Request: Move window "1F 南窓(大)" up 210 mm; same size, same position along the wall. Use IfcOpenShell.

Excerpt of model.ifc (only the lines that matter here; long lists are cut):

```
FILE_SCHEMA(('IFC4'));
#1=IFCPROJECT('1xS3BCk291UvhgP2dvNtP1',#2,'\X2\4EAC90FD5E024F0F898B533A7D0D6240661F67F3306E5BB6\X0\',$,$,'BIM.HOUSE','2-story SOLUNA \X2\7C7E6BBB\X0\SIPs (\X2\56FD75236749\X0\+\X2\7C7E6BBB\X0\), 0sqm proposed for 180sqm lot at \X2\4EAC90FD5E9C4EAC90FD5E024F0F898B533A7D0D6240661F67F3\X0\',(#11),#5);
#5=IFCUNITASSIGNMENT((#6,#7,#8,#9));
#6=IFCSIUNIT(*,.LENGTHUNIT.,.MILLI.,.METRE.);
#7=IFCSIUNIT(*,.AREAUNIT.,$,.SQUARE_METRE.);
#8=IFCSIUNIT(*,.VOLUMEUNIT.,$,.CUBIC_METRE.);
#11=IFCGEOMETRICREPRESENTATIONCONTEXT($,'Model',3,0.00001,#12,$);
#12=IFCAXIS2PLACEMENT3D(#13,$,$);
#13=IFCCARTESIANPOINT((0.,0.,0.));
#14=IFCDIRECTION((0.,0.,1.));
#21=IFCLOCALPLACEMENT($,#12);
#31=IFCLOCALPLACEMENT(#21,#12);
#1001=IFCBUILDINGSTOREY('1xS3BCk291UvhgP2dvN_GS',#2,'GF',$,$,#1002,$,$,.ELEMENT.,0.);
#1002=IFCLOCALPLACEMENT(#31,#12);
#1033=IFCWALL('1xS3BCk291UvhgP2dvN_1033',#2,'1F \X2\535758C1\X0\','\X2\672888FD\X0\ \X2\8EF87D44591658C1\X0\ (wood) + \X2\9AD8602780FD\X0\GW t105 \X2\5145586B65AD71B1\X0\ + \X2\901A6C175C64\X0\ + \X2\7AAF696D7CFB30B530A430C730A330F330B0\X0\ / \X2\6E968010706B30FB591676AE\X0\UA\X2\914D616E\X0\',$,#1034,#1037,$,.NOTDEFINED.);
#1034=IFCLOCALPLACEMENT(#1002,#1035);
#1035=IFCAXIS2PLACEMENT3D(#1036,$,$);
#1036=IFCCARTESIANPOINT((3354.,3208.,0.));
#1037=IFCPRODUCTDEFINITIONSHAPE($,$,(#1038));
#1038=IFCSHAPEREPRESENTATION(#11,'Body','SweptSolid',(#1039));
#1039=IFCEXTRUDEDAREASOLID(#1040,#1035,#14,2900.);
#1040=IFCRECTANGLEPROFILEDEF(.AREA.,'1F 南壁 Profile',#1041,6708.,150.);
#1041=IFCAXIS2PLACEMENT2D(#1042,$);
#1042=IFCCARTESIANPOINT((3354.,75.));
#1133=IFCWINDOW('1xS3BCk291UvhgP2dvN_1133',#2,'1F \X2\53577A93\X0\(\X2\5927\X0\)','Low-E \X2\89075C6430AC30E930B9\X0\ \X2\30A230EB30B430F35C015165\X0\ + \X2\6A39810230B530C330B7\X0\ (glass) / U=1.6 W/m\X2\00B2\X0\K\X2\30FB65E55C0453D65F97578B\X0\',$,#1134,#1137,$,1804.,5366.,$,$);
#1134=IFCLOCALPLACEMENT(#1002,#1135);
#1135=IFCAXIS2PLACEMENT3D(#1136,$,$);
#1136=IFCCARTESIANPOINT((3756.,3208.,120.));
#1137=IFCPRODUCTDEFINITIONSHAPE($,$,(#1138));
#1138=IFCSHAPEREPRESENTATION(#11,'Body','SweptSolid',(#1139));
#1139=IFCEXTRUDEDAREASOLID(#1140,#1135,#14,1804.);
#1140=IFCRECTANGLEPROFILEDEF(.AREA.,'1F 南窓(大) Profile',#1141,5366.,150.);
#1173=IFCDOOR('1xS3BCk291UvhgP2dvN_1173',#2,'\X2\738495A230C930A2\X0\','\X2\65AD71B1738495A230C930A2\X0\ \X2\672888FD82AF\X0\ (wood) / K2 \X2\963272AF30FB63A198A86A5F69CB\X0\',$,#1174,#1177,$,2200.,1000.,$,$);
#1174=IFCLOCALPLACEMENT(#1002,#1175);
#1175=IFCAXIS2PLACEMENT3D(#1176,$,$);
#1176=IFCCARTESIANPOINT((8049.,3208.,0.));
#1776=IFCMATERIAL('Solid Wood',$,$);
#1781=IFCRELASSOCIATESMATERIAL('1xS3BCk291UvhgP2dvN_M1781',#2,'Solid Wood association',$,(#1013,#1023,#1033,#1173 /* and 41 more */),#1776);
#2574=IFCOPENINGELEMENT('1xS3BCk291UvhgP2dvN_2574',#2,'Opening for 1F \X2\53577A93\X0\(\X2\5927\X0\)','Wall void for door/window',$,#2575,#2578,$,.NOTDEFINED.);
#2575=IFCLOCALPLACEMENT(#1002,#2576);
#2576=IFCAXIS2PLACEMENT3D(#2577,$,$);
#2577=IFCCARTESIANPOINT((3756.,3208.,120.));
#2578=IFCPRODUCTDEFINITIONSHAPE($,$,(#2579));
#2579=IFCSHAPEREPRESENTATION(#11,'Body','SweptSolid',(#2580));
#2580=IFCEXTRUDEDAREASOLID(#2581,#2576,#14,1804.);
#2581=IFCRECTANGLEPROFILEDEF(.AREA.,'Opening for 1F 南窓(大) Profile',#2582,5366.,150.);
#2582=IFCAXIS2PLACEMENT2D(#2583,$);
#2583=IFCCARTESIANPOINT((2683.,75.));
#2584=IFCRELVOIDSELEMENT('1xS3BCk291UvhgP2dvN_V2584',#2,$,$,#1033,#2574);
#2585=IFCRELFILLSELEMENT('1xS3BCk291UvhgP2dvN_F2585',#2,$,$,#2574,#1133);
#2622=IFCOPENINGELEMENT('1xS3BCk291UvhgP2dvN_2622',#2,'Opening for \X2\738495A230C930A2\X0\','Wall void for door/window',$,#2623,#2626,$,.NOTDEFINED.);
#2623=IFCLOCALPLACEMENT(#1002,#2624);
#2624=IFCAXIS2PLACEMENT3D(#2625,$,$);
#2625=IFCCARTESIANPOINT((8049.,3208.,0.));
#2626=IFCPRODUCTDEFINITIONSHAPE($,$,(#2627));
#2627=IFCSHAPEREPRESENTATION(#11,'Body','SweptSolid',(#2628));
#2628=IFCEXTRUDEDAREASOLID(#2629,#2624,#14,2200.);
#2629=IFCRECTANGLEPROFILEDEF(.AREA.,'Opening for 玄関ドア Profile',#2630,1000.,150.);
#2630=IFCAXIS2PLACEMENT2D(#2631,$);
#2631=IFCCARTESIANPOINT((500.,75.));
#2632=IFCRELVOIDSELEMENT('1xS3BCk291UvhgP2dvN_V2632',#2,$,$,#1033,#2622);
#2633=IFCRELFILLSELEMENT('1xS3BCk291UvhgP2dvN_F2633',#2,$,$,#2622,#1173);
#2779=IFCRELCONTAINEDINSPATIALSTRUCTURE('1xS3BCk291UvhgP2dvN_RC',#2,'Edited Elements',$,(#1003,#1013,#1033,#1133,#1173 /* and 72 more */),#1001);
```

```python
import numpy as np
import ifcopenshell
import ifcopenshell.api.geometry
import ifcopenshell.util.placement
import ifcopenshell.util.unit

model = ifcopenshell.open("model.ifc")
unit_scale = ifcopenshell.util.unit.calculate_unit_scale(model)

window = model.by_id(1133)
opening = window.FillsVoids[0].RelatingOpeningElement
dz = 0.21 / unit_scale

shift = np.array([0.0, 0.0, dz])
# The window is not placed relative to its opening, so move both.
for product in (opening, window):
    matrix = ifcopenshell.util.placement.get_local_placement(product.ObjectPlacement)
    matrix[:3, 3] += shift
    ifcopenshell.api.geometry.edit_object_placement(model, product=product, matrix=matrix, is_si=False)

print(f"moved by {dz * unit_scale:+.3f} m")

model.write("model_updated.ifc")
```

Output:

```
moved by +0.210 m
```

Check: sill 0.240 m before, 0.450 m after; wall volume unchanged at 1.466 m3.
